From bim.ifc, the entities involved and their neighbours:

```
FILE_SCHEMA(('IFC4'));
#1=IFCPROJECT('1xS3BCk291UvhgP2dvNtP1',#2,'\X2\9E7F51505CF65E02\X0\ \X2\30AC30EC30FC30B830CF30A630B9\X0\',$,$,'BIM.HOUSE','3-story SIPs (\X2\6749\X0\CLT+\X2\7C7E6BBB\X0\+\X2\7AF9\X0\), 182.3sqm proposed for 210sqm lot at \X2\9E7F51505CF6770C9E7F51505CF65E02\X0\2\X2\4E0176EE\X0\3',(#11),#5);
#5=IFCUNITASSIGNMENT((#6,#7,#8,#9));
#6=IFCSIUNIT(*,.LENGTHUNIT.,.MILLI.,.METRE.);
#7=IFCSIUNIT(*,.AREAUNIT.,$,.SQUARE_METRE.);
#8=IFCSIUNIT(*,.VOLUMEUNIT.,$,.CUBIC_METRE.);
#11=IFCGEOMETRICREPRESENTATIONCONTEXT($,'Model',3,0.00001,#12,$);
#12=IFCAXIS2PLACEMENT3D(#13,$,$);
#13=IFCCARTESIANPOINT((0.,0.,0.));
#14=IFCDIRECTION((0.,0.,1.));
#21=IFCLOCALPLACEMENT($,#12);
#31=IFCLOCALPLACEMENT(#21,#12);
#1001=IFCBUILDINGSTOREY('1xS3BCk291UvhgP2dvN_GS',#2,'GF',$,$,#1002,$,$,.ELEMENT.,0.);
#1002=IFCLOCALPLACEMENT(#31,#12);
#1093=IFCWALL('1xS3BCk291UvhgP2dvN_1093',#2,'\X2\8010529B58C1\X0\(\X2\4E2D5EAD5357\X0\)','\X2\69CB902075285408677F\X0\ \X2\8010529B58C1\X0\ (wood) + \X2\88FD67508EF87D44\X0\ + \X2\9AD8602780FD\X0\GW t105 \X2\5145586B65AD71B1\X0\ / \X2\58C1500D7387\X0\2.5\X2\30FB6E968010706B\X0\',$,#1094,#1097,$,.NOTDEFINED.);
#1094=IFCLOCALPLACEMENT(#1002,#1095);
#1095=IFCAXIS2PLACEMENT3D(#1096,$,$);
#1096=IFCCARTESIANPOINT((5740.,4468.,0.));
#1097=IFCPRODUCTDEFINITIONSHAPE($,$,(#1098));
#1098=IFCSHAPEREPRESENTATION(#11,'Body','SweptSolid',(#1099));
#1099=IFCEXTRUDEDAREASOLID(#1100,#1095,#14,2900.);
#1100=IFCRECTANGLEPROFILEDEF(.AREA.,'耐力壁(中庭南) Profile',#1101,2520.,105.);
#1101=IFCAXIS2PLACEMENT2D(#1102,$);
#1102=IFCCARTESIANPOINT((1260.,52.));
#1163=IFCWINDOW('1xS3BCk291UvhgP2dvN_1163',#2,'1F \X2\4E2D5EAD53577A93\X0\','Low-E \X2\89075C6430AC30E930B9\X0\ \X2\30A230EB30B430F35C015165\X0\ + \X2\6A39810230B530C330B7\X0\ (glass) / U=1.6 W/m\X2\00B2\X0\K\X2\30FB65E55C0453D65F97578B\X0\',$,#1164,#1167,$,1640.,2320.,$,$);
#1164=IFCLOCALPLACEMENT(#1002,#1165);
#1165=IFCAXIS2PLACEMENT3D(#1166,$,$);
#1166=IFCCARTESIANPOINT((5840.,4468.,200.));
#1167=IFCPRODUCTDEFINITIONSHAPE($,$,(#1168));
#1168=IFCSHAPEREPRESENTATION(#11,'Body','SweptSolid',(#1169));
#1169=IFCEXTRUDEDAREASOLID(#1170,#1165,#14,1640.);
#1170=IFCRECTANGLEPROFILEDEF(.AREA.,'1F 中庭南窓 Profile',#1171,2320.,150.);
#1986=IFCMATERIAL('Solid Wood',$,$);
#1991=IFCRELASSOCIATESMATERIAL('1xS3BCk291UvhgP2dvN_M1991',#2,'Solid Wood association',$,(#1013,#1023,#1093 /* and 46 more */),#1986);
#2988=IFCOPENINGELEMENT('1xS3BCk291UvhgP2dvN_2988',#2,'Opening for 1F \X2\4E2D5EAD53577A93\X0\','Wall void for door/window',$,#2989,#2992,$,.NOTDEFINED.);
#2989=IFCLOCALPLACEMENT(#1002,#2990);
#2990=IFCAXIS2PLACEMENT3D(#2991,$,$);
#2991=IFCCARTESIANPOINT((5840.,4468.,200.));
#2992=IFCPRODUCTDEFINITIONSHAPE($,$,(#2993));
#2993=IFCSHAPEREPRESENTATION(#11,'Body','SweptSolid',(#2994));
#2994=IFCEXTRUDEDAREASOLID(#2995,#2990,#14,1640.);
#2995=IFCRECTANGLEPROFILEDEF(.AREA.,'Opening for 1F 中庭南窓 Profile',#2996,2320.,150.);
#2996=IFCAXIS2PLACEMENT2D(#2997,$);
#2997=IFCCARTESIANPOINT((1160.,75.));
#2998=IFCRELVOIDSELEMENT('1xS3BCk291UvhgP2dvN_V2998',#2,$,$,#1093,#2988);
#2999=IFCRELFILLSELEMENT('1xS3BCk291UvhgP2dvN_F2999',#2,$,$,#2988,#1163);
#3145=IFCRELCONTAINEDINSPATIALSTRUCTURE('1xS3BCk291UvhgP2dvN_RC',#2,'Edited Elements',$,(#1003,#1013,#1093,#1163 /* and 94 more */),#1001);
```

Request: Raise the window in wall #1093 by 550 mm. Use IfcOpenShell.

```python
import numpy as np
import ifcopenshell
import ifcopenshell.api.geometry
import ifcopenshell.util.placement
import ifcopenshell.util.unit

model = ifcopenshell.open("bim.ifc")
unit_scale = ifcopenshell.util.unit.calculate_unit_scale(model)

window = model.by_guid("1xS3BCk291UvhgP2dvN_1163")
opening = window.FillsVoids[0].RelatingOpeningElement
dz = 0.55 / unit_scale

shift = np.array([0.0, 0.0, dz])
# The window is not placed relative to its opening, so move both.
for product in (opening, window):
    matrix = ifcopenshell.util.placement.get_local_placement(product.ObjectPlacement)
    matrix[:3, 3] += shift
    ifcopenshell.api.geometry.edit_object_placement(model, product=product, matrix=matrix, is_si=False)

print(f"moved by {dz * unit_scale:+.3f} m")

model.write("bim_v2.ifc")
```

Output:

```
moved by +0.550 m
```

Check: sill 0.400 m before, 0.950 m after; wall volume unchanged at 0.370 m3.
